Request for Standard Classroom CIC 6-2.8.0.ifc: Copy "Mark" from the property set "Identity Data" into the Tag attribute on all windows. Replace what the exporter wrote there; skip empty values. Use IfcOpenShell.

First a look at what the model holds.

```python
import ifcopenshell
import ifcopenshell.util.element

model = ifcopenshell.open("Standard Classroom CIC 6-2.8.0.ifc")
print(model.schema)
windows = model.by_type("IfcWindow")
print(len(windows), "windows")
for e in windows[:8]:
    source = ifcopenshell.util.element.get_pset(e, "Identity Data", "Mark")
    target = e.Tag
    print(e.id(), repr(source), repr(target), sep=" | ")
```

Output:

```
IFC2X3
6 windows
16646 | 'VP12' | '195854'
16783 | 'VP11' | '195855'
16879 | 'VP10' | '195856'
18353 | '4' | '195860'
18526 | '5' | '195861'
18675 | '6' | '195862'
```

```python
import ifcopenshell
import ifcopenshell.util.element

model = ifcopenshell.open("Standard Classroom CIC 6-2.8.0.ifc")

count = 0
for e in model.by_type("IfcWindow"):
    value = ifcopenshell.util.element.get_pset(e, "Identity Data", "Mark")
    current = e.Tag
    if not value or not value.strip() or current == value:
        continue
    e.Tag = value
    count += 1

print(count, "windows updated")

model.write("Standard Classroom CIC 6-2.8.0-out.ifc")
```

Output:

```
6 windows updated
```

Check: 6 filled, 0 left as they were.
